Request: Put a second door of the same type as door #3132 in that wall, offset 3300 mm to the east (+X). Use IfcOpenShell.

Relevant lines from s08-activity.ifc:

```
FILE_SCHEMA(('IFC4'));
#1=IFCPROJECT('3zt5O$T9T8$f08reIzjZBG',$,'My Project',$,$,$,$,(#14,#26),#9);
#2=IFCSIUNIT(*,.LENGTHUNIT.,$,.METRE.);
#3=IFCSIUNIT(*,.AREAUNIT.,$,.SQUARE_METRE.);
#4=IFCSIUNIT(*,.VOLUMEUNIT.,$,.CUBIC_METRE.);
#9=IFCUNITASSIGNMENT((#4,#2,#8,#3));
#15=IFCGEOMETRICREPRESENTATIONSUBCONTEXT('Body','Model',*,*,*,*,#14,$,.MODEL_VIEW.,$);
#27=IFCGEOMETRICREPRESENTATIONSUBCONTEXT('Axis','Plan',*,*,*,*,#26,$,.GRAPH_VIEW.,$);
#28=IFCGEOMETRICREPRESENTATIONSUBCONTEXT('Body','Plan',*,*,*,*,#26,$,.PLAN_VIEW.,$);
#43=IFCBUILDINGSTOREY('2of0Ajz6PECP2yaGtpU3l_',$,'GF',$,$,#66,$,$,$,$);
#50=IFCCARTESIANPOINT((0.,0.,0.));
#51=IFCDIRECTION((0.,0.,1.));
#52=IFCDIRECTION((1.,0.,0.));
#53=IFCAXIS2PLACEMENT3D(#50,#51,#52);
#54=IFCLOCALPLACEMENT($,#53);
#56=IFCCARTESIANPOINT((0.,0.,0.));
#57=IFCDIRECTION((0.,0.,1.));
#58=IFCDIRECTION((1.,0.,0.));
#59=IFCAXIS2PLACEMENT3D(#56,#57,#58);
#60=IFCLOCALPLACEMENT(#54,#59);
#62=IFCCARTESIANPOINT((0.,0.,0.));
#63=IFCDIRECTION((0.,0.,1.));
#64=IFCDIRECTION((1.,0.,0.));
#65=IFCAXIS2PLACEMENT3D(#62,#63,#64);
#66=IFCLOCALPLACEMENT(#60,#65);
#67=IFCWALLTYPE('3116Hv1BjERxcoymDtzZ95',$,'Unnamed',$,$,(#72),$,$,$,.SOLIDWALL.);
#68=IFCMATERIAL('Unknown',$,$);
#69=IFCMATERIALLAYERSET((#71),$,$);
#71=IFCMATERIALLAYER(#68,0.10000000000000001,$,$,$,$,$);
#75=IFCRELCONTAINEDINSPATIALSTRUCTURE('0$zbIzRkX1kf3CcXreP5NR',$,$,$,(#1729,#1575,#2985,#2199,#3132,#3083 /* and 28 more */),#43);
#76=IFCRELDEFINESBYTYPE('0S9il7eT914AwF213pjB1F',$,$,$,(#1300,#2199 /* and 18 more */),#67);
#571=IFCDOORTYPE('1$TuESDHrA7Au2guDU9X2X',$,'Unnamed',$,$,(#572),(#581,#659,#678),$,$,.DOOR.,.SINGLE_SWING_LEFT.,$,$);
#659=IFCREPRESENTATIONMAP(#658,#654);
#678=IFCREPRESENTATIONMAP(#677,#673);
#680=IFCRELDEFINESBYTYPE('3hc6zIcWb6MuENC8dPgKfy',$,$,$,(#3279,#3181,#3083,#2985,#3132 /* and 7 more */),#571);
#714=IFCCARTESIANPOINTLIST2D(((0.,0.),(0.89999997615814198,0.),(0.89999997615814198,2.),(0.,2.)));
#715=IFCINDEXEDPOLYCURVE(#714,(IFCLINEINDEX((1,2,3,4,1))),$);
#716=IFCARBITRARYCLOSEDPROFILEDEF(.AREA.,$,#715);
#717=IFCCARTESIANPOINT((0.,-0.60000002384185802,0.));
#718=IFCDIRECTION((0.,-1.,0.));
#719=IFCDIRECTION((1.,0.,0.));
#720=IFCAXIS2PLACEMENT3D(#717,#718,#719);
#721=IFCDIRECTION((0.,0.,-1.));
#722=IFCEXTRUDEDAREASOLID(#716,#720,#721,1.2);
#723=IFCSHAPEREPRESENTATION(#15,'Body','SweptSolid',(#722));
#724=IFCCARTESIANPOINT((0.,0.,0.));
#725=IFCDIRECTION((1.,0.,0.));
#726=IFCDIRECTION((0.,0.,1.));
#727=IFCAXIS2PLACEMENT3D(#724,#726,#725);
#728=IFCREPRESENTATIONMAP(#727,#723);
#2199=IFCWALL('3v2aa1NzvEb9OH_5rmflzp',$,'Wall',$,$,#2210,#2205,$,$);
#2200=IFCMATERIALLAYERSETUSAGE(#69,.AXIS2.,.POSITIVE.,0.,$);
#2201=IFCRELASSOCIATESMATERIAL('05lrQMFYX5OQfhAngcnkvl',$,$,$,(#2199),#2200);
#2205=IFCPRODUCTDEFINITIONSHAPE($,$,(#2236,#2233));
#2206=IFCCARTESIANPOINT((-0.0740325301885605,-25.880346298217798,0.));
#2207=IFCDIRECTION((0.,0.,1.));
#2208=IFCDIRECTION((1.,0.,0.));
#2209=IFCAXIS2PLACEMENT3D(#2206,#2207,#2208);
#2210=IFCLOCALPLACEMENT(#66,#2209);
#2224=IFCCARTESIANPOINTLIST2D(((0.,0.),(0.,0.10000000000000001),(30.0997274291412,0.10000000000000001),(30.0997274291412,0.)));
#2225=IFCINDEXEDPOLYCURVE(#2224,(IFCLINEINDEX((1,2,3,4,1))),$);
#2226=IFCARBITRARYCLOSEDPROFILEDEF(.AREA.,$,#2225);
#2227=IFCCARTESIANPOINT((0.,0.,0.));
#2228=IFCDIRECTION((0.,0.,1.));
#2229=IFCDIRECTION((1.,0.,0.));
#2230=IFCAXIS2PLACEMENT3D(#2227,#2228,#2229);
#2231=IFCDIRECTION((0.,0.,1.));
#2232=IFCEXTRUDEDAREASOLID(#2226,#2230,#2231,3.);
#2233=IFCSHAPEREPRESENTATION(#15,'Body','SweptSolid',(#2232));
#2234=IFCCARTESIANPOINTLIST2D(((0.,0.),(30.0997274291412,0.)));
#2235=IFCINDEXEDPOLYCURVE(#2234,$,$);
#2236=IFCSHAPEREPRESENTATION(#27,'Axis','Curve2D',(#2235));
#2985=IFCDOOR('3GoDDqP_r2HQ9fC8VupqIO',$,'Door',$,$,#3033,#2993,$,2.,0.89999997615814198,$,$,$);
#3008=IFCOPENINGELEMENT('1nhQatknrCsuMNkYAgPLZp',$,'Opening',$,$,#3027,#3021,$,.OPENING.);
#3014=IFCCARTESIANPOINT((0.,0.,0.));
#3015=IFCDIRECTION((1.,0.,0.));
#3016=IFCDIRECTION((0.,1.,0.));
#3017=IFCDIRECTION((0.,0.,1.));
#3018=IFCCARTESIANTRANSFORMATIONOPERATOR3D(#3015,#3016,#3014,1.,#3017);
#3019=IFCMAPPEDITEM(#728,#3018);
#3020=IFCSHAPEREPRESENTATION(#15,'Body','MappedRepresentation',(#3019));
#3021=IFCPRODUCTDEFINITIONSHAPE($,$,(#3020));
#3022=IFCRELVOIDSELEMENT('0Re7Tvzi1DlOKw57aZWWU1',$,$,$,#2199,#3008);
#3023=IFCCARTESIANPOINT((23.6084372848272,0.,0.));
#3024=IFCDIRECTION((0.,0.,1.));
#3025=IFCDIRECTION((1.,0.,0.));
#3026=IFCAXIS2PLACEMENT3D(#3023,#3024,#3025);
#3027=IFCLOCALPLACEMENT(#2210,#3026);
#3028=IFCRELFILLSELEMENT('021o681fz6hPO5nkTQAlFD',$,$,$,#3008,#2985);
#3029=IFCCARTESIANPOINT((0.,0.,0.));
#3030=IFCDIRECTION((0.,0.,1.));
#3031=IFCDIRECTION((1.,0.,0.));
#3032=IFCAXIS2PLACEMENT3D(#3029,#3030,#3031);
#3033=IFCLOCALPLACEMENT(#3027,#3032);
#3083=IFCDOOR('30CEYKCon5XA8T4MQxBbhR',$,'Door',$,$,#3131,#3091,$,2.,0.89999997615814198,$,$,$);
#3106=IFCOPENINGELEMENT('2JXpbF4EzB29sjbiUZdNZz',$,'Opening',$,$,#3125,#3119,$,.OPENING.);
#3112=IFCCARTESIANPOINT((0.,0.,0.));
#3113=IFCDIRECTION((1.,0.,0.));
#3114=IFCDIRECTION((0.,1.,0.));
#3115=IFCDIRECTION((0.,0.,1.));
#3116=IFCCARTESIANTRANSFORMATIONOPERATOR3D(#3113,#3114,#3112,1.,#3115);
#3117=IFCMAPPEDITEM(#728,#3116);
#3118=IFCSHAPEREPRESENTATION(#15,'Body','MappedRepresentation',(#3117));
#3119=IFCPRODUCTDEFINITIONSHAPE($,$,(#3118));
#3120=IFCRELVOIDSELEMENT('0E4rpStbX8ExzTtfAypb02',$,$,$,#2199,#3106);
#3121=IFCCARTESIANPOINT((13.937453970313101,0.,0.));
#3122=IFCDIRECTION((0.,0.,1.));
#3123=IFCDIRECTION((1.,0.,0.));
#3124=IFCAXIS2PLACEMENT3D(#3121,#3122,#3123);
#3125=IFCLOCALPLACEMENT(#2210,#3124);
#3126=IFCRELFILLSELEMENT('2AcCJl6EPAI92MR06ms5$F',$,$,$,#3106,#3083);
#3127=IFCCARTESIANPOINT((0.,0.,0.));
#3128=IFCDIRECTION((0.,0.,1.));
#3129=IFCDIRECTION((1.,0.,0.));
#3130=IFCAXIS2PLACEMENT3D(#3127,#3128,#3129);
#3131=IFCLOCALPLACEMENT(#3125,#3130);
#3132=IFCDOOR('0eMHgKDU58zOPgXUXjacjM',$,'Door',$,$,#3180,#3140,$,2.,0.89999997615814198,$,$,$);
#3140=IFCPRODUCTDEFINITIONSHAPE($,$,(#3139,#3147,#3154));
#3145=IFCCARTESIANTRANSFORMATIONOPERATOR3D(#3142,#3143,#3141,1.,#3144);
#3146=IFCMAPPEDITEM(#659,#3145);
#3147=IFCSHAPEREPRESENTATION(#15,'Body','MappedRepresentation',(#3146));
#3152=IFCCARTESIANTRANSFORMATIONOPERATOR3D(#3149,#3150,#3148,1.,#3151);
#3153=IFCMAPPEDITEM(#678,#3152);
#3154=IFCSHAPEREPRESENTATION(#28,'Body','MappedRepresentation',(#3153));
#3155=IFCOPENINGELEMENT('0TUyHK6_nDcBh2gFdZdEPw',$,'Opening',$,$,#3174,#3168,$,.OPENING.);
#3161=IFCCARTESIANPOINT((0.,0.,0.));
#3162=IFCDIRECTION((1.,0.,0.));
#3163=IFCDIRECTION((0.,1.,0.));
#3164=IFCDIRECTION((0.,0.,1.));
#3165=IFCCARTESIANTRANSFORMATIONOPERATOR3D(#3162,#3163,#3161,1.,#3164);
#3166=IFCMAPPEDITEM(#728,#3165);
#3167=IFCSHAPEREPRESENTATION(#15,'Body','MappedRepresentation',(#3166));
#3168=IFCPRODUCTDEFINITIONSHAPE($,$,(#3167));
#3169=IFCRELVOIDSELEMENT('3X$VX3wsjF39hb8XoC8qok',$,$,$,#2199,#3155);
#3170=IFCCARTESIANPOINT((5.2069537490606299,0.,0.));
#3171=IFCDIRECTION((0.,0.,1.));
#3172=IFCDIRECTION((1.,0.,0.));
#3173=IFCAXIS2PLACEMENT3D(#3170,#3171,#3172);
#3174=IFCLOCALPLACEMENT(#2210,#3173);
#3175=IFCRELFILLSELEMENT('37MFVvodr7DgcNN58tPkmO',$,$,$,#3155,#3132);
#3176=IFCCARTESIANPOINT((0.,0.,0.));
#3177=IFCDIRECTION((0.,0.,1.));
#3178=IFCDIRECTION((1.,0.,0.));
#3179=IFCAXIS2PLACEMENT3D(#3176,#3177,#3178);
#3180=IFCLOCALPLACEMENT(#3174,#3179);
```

```python
import ifcopenshell
import ifcopenshell.api.feature
import ifcopenshell.api.geometry
import ifcopenshell.api.root
import ifcopenshell.geom
import ifcopenshell.util.element
import ifcopenshell.util.placement
import ifcopenshell.util.shape
import ifcopenshell.util.unit

model = ifcopenshell.open("s08-activity.ifc")
unit_scale = ifcopenshell.util.unit.calculate_unit_scale(model)
settings = ifcopenshell.geom.settings()


def volume(element):
    """Net volume in cubic metres, openings subtracted."""
    shape = ifcopenshell.geom.create_shape(settings, element)
    return ifcopenshell.util.shape.get_volume(shape.geometry)


door = model.by_guid("0eMHgKDU58zOPgXUXjacjM")
opening = door.FillsVoids[0].RelatingOpeningElement
wall = opening.VoidsElements[0].RelatingBuildingElement
before = volume(wall)
shift = ifcopenshell.util.placement.get_local_placement(wall.ObjectPlacement)[:3, 0] * 3.3 / unit_scale

# copy_class copies the void relationship, type, container and properties, but no geometry.
new_opening = ifcopenshell.api.root.copy_class(model, product=opening)
new_opening.Representation = ifcopenshell.util.element.copy_deep(
    model, opening.Representation, exclude=["IfcGeometricRepresentationContext", "IfcRepresentationMap"]
)
new_door = ifcopenshell.api.root.copy_class(model, product=door)
new_door.Representation = ifcopenshell.util.element.copy_deep(
    model, door.Representation, exclude=["IfcGeometricRepresentationContext", "IfcRepresentationMap"]
)
ifcopenshell.api.feature.add_filling(model, opening=new_opening, element=new_door)

for old, new in ((opening, new_opening), (door, new_door)):
    matrix = ifcopenshell.util.placement.get_local_placement(old.ObjectPlacement)
    matrix[:3, 3] += shift
    ifcopenshell.api.geometry.edit_object_placement(model, product=new, matrix=matrix, is_si=False)

after = volume(wall)

print(f"wall volume {before:.3f} -> {after:.3f} m3")

model.write("s08-activity_edited.ifc")
```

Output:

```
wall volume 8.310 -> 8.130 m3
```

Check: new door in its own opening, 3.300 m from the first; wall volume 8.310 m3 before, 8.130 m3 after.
